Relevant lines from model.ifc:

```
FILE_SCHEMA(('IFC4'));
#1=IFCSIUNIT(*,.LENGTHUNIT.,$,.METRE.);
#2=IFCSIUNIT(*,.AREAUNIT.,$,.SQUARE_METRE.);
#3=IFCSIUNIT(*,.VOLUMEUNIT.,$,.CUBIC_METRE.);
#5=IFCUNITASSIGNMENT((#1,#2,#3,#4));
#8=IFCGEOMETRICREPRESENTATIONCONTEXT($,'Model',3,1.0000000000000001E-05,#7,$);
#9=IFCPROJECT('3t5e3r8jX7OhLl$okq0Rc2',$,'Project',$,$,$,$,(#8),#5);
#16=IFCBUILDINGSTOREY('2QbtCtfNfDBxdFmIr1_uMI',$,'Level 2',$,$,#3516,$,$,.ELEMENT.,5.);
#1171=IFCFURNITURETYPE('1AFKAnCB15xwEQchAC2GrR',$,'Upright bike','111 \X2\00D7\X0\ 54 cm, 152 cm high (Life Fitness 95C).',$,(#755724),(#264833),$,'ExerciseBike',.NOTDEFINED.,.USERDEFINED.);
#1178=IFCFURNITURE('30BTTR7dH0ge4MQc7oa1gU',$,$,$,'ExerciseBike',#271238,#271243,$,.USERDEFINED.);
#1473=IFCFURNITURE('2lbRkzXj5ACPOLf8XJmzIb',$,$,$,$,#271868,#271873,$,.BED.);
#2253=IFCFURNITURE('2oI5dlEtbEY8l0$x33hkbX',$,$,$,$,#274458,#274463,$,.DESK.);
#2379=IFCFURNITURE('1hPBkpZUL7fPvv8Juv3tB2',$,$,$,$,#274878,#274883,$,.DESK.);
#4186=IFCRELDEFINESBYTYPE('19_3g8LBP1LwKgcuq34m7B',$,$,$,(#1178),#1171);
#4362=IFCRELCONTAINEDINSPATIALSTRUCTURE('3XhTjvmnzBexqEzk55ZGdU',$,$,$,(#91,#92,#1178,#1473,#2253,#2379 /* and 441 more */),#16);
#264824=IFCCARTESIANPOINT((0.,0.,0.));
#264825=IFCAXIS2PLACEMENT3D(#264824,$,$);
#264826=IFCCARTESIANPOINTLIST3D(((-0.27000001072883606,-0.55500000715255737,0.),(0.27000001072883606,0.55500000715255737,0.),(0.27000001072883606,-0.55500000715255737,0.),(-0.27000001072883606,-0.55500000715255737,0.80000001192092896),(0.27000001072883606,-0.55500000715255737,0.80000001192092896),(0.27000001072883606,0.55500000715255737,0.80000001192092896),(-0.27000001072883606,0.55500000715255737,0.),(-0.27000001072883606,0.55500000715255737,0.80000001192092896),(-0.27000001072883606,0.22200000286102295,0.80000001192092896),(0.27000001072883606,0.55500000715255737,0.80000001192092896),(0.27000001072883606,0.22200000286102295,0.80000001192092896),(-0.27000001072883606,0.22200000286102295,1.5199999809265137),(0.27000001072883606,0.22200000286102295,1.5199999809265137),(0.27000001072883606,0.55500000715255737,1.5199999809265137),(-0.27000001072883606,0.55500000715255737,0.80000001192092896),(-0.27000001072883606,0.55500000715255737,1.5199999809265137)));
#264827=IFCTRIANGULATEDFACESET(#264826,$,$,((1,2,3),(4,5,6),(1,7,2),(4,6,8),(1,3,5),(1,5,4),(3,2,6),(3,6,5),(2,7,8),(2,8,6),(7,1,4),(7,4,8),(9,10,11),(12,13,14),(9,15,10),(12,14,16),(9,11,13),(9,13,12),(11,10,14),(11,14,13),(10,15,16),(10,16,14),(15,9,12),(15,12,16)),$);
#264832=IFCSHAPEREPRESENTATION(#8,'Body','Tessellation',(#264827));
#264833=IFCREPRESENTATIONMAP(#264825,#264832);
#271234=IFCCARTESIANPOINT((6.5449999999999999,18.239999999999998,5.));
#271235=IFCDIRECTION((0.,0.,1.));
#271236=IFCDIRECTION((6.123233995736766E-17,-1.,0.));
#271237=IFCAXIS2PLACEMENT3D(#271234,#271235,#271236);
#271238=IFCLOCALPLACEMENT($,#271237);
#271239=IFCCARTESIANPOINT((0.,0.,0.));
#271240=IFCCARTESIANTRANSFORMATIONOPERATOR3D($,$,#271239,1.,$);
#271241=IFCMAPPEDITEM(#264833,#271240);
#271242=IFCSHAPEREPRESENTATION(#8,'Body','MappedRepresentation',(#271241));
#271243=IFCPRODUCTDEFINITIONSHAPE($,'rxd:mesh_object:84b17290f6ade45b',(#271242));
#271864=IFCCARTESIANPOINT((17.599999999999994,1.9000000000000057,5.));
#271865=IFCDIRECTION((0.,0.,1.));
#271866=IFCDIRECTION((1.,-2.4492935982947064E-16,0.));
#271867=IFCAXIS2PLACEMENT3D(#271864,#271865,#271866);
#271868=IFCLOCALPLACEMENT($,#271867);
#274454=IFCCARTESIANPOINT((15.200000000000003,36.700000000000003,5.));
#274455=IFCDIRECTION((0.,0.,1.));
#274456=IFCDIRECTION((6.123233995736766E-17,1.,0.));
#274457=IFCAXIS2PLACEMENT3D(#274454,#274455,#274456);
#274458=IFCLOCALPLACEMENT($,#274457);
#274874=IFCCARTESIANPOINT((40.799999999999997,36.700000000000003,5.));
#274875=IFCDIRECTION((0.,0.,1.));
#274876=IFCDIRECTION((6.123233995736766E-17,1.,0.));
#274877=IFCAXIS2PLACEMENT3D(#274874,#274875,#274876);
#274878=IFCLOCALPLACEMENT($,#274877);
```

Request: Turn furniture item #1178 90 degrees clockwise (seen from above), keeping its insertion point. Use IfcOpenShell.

```python
import ifcopenshell
import ifcopenshell.api.geometry
import ifcopenshell.util.placement

model = ifcopenshell.open("model.ifc")

item = model.by_guid("30BTTR7dH0ge4MQc7oa1gU")
matrix = ifcopenshell.util.placement.get_local_placement(item.ObjectPlacement)
matrix = matrix @ ifcopenshell.util.placement.rotation(-90, "Z")
ifcopenshell.api.geometry.edit_object_placement(model, product=item, matrix=matrix, is_si=False)

print(ifcopenshell.util.placement.get_local_placement(item.ObjectPlacement).round(3) + 0.0)

model.write("model_edited.ifc")
```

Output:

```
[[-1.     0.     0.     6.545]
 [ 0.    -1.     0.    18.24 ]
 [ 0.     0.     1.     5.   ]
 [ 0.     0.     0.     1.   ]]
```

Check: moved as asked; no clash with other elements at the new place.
